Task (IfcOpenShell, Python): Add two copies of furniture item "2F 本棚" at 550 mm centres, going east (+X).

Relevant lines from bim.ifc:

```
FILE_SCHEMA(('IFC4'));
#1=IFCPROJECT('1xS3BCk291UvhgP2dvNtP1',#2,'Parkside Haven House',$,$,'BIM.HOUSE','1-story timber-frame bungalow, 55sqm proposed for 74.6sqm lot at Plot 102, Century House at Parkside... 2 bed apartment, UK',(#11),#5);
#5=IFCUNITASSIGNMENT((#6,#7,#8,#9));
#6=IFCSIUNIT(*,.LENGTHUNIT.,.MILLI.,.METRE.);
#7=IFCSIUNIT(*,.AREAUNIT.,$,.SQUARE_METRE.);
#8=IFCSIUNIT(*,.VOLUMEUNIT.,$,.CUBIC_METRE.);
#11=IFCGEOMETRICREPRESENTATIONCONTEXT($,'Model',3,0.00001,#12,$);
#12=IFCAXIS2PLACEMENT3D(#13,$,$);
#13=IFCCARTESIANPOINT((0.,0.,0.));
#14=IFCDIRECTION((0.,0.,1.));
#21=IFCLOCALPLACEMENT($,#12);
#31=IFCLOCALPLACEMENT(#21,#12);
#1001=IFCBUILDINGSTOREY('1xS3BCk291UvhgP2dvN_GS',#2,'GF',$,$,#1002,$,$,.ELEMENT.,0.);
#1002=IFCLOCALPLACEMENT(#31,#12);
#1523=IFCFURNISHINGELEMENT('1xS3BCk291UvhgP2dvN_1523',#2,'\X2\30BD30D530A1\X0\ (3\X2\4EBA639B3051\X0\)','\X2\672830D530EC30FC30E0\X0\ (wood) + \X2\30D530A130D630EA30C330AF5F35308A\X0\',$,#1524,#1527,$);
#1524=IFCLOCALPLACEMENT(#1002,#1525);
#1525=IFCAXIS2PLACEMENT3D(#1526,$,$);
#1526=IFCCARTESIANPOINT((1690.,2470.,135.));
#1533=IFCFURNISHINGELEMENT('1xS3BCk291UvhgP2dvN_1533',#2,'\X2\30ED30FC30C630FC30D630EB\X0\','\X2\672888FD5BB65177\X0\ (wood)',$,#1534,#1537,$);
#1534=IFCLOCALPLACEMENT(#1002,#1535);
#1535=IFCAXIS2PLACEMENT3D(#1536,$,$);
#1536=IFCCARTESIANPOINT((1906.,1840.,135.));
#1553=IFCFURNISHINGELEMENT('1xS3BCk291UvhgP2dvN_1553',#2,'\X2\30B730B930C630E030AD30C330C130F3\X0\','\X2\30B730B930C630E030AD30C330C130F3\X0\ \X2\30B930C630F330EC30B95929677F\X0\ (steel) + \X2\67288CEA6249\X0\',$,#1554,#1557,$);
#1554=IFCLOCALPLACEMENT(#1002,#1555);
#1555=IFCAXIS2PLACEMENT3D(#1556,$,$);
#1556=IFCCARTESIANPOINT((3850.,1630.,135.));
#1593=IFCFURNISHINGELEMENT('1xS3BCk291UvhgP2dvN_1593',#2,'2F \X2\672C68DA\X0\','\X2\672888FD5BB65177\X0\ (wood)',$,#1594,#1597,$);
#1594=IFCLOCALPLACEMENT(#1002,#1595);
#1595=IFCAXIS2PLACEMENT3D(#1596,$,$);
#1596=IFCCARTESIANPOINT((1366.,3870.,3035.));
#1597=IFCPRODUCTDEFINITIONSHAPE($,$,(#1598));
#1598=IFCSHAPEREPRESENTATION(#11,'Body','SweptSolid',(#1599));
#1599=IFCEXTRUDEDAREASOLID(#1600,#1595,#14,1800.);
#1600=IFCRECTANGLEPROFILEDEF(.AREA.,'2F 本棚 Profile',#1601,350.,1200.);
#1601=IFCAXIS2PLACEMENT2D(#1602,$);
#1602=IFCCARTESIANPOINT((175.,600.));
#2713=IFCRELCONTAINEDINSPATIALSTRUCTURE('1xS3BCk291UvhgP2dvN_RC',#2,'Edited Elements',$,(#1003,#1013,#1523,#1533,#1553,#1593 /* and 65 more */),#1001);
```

```python
import numpy as np
import ifcopenshell
import ifcopenshell.api.geometry
import ifcopenshell.api.root
import ifcopenshell.util.element
import ifcopenshell.util.placement
import ifcopenshell.util.unit

model = ifcopenshell.open("bim.ifc")
unit_scale = ifcopenshell.util.unit.calculate_unit_scale(model)


def reuse_history(source, copy):
    """copy_class also copies each property set's owner history, people and application; keep the originals."""
    for rel in copy.IsDefinedBy:
        if rel.is_a("IfcRelDefinesByProperties") and (history := rel.RelatingPropertyDefinition.OwnerHistory):
            rel.RelatingPropertyDefinition.OwnerHistory = source.OwnerHistory
            ifcopenshell.util.element.remove_deep2(model, history)


source = model.by_guid("1xS3BCk291UvhgP2dvN_1593")
base = ifcopenshell.util.placement.get_local_placement(source.ObjectPlacement)
step = np.array([1.0, 0.0, 0.0]) * 0.55 / unit_scale

for i in range(1, 3):
    copy = ifcopenshell.api.root.copy_class(model, product=source)
    copy.Representation = ifcopenshell.util.element.copy_deep(
        model, source.Representation, exclude=["IfcGeometricRepresentationContext", "IfcRepresentationMap"]
    )
    reuse_history(source, copy)
    matrix = base.copy()
    matrix[:3, 3] += i * step
    print("added at", matrix[:3, 3].round(3) + 0.0)
    ifcopenshell.api.geometry.edit_object_placement(model, product=copy, matrix=matrix, is_si=False)

model.write("bim_edited.ifc")
```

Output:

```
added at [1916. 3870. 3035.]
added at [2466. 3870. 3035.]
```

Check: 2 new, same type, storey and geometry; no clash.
